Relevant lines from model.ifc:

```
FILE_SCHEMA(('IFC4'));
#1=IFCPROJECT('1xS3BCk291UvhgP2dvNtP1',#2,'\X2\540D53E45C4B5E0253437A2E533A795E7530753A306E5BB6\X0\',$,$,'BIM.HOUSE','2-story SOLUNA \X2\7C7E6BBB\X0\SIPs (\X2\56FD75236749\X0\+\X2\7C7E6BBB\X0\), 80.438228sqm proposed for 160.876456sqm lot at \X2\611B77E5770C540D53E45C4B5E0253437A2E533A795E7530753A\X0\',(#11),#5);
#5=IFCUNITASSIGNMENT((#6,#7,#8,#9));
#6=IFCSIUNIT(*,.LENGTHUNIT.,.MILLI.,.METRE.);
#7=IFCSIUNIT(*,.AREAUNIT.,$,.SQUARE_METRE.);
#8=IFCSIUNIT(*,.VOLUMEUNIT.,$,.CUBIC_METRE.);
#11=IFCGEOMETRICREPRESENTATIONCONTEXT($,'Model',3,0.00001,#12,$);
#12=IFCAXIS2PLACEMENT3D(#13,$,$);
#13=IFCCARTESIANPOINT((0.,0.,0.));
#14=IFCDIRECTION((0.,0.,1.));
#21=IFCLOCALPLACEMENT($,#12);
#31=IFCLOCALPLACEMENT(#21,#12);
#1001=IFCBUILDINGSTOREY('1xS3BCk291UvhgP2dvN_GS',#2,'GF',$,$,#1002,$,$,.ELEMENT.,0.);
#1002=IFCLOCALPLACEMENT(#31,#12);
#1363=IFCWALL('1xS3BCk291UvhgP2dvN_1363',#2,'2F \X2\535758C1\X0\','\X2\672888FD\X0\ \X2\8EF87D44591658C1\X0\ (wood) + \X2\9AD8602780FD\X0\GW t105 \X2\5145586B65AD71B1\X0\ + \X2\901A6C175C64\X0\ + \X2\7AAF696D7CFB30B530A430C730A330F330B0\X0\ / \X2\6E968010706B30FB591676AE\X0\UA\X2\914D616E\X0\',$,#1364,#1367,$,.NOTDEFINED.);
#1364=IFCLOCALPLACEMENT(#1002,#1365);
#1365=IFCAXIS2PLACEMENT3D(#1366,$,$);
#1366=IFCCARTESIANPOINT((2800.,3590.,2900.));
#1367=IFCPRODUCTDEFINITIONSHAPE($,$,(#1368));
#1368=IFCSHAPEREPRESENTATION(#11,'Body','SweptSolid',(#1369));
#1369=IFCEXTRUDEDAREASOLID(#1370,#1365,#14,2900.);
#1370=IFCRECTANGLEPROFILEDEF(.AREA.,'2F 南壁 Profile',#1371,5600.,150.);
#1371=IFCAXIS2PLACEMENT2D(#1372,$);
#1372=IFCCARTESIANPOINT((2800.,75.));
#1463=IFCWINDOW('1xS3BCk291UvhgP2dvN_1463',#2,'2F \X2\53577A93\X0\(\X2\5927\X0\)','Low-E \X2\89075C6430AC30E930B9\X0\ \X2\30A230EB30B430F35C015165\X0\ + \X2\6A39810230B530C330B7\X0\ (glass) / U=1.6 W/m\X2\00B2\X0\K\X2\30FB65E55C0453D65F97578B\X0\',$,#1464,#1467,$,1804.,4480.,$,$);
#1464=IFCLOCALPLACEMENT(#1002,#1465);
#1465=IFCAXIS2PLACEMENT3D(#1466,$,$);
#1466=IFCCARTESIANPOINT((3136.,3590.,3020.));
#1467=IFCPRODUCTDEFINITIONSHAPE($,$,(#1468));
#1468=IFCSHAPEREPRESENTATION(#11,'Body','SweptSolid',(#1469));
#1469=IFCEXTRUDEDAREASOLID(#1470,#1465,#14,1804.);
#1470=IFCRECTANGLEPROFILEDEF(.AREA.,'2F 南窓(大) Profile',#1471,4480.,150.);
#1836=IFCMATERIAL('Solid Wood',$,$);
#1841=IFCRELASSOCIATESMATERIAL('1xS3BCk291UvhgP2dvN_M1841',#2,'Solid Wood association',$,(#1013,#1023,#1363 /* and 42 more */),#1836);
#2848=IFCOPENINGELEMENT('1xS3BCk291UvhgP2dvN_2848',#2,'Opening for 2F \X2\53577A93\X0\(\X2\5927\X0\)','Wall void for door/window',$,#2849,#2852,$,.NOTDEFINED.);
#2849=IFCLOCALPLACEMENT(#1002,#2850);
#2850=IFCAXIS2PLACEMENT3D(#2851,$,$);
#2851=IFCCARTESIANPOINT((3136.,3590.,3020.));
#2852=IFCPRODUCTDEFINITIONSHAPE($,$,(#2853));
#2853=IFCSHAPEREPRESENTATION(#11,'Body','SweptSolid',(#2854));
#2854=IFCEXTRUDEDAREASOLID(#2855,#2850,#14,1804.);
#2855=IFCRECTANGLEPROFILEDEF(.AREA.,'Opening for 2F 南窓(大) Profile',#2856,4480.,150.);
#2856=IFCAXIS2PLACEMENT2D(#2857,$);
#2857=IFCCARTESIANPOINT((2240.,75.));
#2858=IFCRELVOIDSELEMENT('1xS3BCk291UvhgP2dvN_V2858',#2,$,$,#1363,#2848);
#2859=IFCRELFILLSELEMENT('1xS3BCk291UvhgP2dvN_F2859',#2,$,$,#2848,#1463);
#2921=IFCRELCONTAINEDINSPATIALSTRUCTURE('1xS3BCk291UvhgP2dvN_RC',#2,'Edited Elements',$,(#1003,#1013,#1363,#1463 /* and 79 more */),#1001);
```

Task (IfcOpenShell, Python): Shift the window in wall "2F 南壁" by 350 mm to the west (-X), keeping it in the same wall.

```python
import ifcopenshell
import ifcopenshell.api.geometry
import ifcopenshell.util.placement
import ifcopenshell.util.unit

model = ifcopenshell.open("model.ifc")
unit_scale = ifcopenshell.util.unit.calculate_unit_scale(model)

window = model.by_guid("1xS3BCk291UvhgP2dvN_1463")
opening = window.FillsVoids[0].RelatingOpeningElement
wall = opening.VoidsElements[0].RelatingBuildingElement

wall_matrix = ifcopenshell.util.placement.get_local_placement(wall.ObjectPlacement)
shift = wall_matrix[:3, 0] * -0.35 / unit_scale
before = ifcopenshell.util.placement.get_local_placement(window.ObjectPlacement)[:3, 3].copy()

# The window is not placed relative to its opening, so move both.
for product in (opening, window):
    matrix = ifcopenshell.util.placement.get_local_placement(product.ObjectPlacement)
    matrix[:3, 3] += shift
    ifcopenshell.api.geometry.edit_object_placement(model, product=product, matrix=matrix, is_si=False)

after = ifcopenshell.util.placement.get_local_placement(window.ObjectPlacement)[:3, 3]
print("window moved by", (after - before).round(3) + 0.0)

model.write("model_rev.ifc")
```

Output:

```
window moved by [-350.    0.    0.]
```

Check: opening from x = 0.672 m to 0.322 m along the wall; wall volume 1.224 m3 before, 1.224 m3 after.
